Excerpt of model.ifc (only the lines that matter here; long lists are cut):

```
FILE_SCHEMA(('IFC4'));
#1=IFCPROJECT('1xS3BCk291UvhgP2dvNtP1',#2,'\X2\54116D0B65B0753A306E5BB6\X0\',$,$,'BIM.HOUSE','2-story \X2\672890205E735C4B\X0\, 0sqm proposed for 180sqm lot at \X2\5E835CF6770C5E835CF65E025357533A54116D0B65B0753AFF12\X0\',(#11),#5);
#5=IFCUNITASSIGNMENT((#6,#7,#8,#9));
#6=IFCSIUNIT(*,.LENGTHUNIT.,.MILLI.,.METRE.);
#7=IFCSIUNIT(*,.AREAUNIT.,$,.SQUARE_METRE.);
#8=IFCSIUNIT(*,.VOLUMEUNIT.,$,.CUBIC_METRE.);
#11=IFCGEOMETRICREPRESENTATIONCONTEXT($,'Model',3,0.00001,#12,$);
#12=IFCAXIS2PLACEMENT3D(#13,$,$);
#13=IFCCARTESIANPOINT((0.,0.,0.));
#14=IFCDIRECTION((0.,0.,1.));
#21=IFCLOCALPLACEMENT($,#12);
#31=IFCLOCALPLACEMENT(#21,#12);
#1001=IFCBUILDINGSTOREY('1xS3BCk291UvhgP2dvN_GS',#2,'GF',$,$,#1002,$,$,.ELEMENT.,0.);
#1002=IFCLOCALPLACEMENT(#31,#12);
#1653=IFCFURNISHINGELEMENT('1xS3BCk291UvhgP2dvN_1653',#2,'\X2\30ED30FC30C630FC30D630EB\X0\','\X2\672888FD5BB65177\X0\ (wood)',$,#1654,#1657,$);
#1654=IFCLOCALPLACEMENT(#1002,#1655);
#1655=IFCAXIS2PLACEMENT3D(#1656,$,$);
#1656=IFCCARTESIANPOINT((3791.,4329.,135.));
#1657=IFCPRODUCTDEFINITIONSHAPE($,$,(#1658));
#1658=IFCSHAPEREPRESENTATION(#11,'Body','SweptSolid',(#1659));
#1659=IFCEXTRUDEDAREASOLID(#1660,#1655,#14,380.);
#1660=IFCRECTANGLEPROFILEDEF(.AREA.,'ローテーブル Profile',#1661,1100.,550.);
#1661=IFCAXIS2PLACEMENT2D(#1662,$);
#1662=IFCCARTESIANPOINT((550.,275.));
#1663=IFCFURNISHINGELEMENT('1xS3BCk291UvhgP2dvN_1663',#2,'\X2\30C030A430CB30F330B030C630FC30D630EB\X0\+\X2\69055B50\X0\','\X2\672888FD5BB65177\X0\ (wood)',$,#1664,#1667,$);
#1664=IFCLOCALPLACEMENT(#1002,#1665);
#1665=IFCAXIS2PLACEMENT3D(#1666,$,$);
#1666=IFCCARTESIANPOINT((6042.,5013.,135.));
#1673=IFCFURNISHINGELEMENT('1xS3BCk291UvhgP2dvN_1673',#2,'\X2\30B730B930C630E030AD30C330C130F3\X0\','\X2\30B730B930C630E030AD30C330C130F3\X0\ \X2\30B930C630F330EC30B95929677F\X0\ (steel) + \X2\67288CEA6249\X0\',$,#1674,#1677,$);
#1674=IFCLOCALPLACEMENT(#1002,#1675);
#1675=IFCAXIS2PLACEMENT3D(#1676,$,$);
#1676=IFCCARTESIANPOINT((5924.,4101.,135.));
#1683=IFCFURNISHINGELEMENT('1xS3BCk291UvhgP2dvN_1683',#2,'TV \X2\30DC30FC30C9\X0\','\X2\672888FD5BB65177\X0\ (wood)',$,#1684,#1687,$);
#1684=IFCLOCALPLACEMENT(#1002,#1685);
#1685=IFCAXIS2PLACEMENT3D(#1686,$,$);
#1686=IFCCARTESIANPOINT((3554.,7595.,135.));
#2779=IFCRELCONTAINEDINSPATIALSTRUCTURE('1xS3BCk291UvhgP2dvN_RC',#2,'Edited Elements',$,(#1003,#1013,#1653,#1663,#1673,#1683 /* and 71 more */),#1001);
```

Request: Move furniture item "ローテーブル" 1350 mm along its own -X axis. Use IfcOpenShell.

```python
import ifcopenshell
import ifcopenshell.api.geometry
import ifcopenshell.util.placement
import ifcopenshell.util.unit

model = ifcopenshell.open("model.ifc")
unit_scale = ifcopenshell.util.unit.calculate_unit_scale(model)

item = model.by_guid("1xS3BCk291UvhgP2dvN_1653")
matrix = ifcopenshell.util.placement.get_local_placement(item.ObjectPlacement)
matrix[:3, 3] -= matrix[:3, 0] * 1.35 / unit_scale
ifcopenshell.api.geometry.edit_object_placement(model, product=item, matrix=matrix, is_si=False)

print(ifcopenshell.util.placement.get_local_placement(item.ObjectPlacement).round(3) + 0.0)

model.write("model-out.ifc")
```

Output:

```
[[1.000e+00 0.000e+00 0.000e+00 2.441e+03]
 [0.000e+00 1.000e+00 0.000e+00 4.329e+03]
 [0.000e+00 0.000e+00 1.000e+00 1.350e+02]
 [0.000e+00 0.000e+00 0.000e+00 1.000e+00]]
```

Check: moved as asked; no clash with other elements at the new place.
